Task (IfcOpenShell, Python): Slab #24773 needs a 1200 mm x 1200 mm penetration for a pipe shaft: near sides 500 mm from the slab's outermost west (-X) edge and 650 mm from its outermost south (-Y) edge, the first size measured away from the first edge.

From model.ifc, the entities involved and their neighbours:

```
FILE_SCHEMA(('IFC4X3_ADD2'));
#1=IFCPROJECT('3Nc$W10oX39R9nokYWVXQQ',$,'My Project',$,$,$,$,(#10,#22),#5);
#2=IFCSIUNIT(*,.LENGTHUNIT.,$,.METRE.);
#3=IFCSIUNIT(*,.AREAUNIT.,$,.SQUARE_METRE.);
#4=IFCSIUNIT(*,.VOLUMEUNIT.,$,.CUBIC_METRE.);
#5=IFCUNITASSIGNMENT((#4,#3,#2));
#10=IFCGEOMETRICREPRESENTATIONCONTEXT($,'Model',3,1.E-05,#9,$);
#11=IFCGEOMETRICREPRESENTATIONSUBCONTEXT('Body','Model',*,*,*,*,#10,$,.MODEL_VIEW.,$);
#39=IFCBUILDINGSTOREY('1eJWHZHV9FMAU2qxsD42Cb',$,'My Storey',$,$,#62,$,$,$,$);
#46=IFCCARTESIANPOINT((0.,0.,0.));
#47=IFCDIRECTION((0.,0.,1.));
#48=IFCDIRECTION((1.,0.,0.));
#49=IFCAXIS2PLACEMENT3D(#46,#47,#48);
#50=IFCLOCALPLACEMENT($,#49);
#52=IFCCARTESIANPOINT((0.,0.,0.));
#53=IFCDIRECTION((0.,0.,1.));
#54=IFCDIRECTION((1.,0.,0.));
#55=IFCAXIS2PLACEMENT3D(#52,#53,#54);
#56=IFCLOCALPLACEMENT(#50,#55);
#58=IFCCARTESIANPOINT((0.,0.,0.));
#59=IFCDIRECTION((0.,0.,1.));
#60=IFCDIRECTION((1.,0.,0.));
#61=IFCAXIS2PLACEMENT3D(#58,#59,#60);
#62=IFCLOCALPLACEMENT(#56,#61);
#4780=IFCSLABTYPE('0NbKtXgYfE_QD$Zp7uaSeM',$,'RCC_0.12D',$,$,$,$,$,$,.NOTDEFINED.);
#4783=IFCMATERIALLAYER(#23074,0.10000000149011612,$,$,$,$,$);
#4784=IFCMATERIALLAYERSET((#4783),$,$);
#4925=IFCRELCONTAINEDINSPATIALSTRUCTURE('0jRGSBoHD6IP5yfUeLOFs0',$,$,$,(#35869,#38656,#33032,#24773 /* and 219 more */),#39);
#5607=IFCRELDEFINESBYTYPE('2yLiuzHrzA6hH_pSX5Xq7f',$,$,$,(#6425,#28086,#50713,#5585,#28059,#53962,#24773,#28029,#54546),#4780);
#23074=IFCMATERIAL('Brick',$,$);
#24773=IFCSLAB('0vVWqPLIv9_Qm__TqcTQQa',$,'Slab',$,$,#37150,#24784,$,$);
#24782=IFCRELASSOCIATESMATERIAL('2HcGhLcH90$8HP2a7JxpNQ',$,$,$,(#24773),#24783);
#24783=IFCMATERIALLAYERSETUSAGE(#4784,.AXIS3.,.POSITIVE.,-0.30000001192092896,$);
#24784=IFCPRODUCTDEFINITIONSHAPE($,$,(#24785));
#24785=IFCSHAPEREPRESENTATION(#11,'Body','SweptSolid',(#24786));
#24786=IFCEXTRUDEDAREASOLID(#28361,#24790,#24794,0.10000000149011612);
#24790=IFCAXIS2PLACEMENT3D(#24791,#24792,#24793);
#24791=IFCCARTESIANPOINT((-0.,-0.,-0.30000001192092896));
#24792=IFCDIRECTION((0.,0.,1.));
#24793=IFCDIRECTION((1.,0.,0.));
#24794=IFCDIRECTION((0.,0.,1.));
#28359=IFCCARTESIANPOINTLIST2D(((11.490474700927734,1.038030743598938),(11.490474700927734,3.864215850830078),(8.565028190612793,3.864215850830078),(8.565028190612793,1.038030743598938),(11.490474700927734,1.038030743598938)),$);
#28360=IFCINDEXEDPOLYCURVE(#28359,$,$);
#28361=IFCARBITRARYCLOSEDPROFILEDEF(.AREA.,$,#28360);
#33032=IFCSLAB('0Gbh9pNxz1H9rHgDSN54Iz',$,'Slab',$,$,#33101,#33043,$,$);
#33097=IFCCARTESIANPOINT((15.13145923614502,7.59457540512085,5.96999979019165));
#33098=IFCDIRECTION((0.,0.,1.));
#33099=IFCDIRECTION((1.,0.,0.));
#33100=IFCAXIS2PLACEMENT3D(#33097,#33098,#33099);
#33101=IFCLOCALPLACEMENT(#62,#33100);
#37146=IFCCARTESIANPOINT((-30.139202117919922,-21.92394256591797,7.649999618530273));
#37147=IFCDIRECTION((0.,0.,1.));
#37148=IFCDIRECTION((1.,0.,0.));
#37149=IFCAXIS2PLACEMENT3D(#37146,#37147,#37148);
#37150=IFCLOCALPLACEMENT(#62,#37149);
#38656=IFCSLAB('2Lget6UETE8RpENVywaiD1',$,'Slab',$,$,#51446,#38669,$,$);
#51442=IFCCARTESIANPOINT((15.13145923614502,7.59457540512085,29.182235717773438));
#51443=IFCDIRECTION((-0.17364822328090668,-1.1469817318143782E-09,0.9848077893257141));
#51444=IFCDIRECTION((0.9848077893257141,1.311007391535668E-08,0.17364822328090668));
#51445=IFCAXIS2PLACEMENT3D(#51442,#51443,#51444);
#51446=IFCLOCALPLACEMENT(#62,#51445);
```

```python
import numpy as np
import ifcopenshell
import ifcopenshell.api.feature
import ifcopenshell.api.geometry
import ifcopenshell.api.root
import ifcopenshell.geom
import ifcopenshell.util.placement
import ifcopenshell.util.representation
import ifcopenshell.util.shape
import ifcopenshell.util.unit

model = ifcopenshell.open("model.ifc")
unit_scale = ifcopenshell.util.unit.calculate_unit_scale(model)
settings = ifcopenshell.geom.settings()


def volume(element):
    """Net volume in cubic metres, openings subtracted."""
    shape = ifcopenshell.geom.create_shape(settings, element)
    return ifcopenshell.util.shape.get_volume(shape.geometry)


slab = model.by_guid("0vVWqPLIv9_Qm__TqcTQQa")
before = volume(slab)

# Extent in the slab's own axes, in metres. The edges named are its -X and -Y sides.
slab_shape = ifcopenshell.geom.create_shape(settings, slab)
vertices = ifcopenshell.util.shape.get_vertices(slab_shape.geometry)
x_min, y_min, bottom = vertices.min(axis=0)
top = vertices[:, 2].max()

opening = ifcopenshell.api.root.create_entity(model, ifc_class="IfcOpeningElement", name="Pipe shaft opening", predefined_type="OPENING")
context = ifcopenshell.util.representation.get_context(model, "Model", "Body", "MODEL_VIEW")
width, depth = 1.2, 1.2
outline = [(0.0, 0.0), (width, 0.0), (width, depth), (0.0, depth), (0.0, 0.0)]
# Overshoot both faces by 50 mm so the cut is clean.
shape = ifcopenshell.api.geometry.add_slab_representation(
    model, context=context, depth=top - bottom + 0.1, polyline=outline
)
ifcopenshell.api.geometry.assign_representation(model, product=opening, representation=shape)

matrix = ifcopenshell.util.placement.get_local_placement(slab.ObjectPlacement)
matrix[:, 3] = matrix @ np.append(np.array([x_min + 0.5, y_min + 0.65, bottom - 0.05]) / unit_scale, 1.0)
ifcopenshell.api.geometry.edit_object_placement(model, product=opening, matrix=matrix, is_si=False)
ifcopenshell.api.feature.add_feature(model, feature=opening, element=slab)

after = volume(slab)

print(f"slab volume {before:.3f} -> {after:.3f} m3")

model.write("model_updated.ifc")
```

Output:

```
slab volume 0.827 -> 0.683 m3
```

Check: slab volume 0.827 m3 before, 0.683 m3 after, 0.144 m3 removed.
